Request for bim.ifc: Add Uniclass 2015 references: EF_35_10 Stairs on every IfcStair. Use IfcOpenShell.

First a look at what the model holds.

```python
import ifcopenshell

model = ifcopenshell.open("bim.ifc")
print(model.schema)
print("classifications:", [c.Name for c in model.by_type("IfcClassification")])
for ifc_class in ("IfcDoor", "IfcRoof", "IfcStair", "IfcWall", "IfcWindow"):
    print(ifc_class, len(model.by_type(ifc_class)))
```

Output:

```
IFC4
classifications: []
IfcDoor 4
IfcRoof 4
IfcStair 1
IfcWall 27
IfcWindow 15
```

```python
import ifcopenshell
import ifcopenshell.api.classification

model = ifcopenshell.open("bim.ifc")

system = ifcopenshell.api.classification.add_classification(model, classification="Uniclass 2015")

codes = {
    "IfcStair": ("EF_35_10", "Stairs"),
}
for ifc_class, (code, name) in codes.items():
    products = model.by_type(ifc_class)
    ifcopenshell.api.classification.add_reference(
        model, products=products, classification=system, identification=code, name=name
    )
    print(code, len(products))

model.write("bim_v2.ifc")
```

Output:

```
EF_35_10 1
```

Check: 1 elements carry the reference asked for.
